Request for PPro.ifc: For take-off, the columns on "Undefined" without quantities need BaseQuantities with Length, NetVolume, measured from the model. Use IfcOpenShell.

First a look at what the model holds.

```python
import ifcopenshell
import ifcopenshell.util.element
import ifcopenshell.util.unit

model = ifcopenshell.open("PPro.ifc")
print(model.schema)
for unit_type in ("LENGTHUNIT", "AREAUNIT", "VOLUMEUNIT"):
    print(unit_type, ifcopenshell.util.unit.calculate_unit_scale(model, unit_type))
storey = next(s for s in model.by_type("IfcBuildingStorey") if s.Name == "Undefined")
columns = [e for e in ifcopenshell.util.element.get_decomposition(storey) if e.is_a("IfcColumn")]
for e in sorted(columns, key=lambda e: e.id()):
    print(e.id(), e.is_a(), e.Name, list(ifcopenshell.util.element.get_psets(e, qtos_only=True)), sep=" | ")
```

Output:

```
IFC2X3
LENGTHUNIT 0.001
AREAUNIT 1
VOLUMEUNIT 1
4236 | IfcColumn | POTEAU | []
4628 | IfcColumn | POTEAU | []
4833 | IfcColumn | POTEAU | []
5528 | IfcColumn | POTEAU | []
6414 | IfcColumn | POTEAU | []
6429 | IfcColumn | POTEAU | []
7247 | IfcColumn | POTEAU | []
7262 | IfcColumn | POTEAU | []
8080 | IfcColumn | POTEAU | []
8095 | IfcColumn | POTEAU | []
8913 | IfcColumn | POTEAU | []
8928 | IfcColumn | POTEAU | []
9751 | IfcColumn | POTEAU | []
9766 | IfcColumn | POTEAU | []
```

```python
import ifcopenshell
import ifcopenshell.api.pset
import ifcopenshell.geom
import ifcopenshell.util.element
import ifcopenshell.util.shape
import ifcopenshell.util.unit

model = ifcopenshell.open("PPro.ifc")
unit_scale = ifcopenshell.util.unit.calculate_unit_scale(model)
volume_scale = ifcopenshell.util.unit.calculate_unit_scale(model, "VOLUMEUNIT")
settings = ifcopenshell.geom.settings()

storey = next(s for s in model.by_type("IfcBuildingStorey") if s.Name == "Undefined")
columns = [e for e in ifcopenshell.util.element.get_decomposition(storey) if e.is_a("IfcColumn")]

for e in sorted(columns, key=lambda e: e.id()):
    if ifcopenshell.util.element.get_psets(e, qtos_only=True, should_inherit=False):
        continue
    # Geometry comes back in metres, in the element's own axes.
    shape = ifcopenshell.geom.create_shape(settings, e)
    values = {
        "Length": ifcopenshell.util.shape.get_z(shape.geometry) / unit_scale,
        "NetVolume": ifcopenshell.util.shape.get_volume(shape.geometry) / volume_scale,
    }
    qto = ifcopenshell.api.pset.add_qto(model, product=e, name="BaseQuantities")
    ifcopenshell.api.pset.edit_qto(model, qto=qto, properties=values)
    print(e.id(), {k: round(v, 3) for k, v in values.items()})

model.write("PPro_updated.ifc")
```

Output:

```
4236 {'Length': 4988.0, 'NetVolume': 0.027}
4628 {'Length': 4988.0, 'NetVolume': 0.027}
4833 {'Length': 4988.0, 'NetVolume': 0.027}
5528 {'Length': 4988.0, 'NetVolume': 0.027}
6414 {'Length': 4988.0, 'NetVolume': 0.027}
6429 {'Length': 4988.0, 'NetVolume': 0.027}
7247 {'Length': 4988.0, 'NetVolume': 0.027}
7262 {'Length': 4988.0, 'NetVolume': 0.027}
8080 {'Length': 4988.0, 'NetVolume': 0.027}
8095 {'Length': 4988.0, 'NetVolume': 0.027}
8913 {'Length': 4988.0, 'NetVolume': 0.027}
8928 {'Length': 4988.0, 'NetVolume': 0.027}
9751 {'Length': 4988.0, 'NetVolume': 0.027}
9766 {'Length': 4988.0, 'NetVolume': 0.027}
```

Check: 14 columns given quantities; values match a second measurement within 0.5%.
